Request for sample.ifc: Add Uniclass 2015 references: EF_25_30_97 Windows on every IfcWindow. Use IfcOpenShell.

First a look at what the model holds.

```python
import ifcopenshell

model = ifcopenshell.open("sample.ifc")
print(model.schema)
print("classifications:", [c.Name for c in model.by_type("IfcClassification")])
for ifc_class in ("IfcDoor", "IfcRoof", "IfcStair", "IfcWall", "IfcWindow"):
    print(ifc_class, len(model.by_type(ifc_class)))
```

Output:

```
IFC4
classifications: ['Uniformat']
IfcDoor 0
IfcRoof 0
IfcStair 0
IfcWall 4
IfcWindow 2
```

```python
import ifcopenshell
import ifcopenshell.api.classification

model = ifcopenshell.open("sample.ifc")

system = ifcopenshell.api.classification.add_classification(model, classification="Uniclass 2015")

codes = {
    "IfcWindow": ("EF_25_30_97", "Windows"),
}
for ifc_class, (code, name) in codes.items():
    products = model.by_type(ifc_class)
    ifcopenshell.api.classification.add_reference(
        model, products=products, classification=system, identification=code, name=name
    )
    print(code, len(products))

model.write("sample_updated.ifc")
```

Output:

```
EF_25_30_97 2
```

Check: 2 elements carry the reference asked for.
